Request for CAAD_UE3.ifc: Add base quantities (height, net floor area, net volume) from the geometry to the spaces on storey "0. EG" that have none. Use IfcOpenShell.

First a look at what the model holds.

```python
import ifcopenshell
import ifcopenshell.util.element
import ifcopenshell.util.unit

model = ifcopenshell.open("CAAD_UE3.ifc")
print(model.schema)
for unit_type in ("LENGTHUNIT", "AREAUNIT", "VOLUMEUNIT"):
    print(unit_type, ifcopenshell.util.unit.calculate_unit_scale(model, unit_type))
storey = next(s for s in model.by_type("IfcBuildingStorey") if s.Name == "0. EG")
spaces = [e for e in ifcopenshell.util.element.get_decomposition(storey) if e.is_a("IfcSpace")]
for e in sorted(spaces, key=lambda e: e.id()):
    print(e.id(), e.is_a(), e.Name, list(ifcopenshell.util.element.get_psets(e, qtos_only=True)), sep=" | ")
```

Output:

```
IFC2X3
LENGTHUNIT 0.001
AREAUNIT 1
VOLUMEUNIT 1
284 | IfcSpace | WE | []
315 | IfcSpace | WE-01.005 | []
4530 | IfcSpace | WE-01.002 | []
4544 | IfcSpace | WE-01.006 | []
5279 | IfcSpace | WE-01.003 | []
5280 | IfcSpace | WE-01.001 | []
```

```python
import ifcopenshell
import ifcopenshell.api.pset
import ifcopenshell.geom
import ifcopenshell.util.element
import ifcopenshell.util.shape
import ifcopenshell.util.unit

model = ifcopenshell.open("CAAD_UE3.ifc")
unit_scale = ifcopenshell.util.unit.calculate_unit_scale(model)
area_scale = ifcopenshell.util.unit.calculate_unit_scale(model, "AREAUNIT")
volume_scale = ifcopenshell.util.unit.calculate_unit_scale(model, "VOLUMEUNIT")
settings = ifcopenshell.geom.settings()

storey = next(s for s in model.by_type("IfcBuildingStorey") if s.Name == "0. EG")
spaces = [e for e in ifcopenshell.util.element.get_decomposition(storey) if e.is_a("IfcSpace")]

for e in sorted(spaces, key=lambda e: e.id()):
    if ifcopenshell.util.element.get_psets(e, qtos_only=True, should_inherit=False):
        continue
    # Geometry comes back in metres, in the element's own axes.
    shape = ifcopenshell.geom.create_shape(settings, e)
    values = {
        "Height": ifcopenshell.util.shape.get_z(shape.geometry) / unit_scale,
        "NetFloorArea": ifcopenshell.util.shape.get_footprint_area(shape.geometry) / area_scale,
        "NetVolume": ifcopenshell.util.shape.get_volume(shape.geometry) / volume_scale,
    }
    qto = ifcopenshell.api.pset.add_qto(model, product=e, name="BaseQuantities")
    ifcopenshell.api.pset.edit_qto(model, qto=qto, properties=values)
    print(e.id(), {k: round(v, 3) for k, v in values.items()})

model.write("CAAD_UE3_rev.ifc")
```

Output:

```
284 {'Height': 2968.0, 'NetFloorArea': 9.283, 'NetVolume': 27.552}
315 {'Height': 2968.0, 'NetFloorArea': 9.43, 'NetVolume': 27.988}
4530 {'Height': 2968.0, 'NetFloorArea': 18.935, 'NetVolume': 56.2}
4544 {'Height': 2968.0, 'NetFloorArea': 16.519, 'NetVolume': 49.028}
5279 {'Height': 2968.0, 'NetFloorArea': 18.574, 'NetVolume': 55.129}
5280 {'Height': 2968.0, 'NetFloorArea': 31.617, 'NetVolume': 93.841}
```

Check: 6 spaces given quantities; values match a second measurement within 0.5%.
